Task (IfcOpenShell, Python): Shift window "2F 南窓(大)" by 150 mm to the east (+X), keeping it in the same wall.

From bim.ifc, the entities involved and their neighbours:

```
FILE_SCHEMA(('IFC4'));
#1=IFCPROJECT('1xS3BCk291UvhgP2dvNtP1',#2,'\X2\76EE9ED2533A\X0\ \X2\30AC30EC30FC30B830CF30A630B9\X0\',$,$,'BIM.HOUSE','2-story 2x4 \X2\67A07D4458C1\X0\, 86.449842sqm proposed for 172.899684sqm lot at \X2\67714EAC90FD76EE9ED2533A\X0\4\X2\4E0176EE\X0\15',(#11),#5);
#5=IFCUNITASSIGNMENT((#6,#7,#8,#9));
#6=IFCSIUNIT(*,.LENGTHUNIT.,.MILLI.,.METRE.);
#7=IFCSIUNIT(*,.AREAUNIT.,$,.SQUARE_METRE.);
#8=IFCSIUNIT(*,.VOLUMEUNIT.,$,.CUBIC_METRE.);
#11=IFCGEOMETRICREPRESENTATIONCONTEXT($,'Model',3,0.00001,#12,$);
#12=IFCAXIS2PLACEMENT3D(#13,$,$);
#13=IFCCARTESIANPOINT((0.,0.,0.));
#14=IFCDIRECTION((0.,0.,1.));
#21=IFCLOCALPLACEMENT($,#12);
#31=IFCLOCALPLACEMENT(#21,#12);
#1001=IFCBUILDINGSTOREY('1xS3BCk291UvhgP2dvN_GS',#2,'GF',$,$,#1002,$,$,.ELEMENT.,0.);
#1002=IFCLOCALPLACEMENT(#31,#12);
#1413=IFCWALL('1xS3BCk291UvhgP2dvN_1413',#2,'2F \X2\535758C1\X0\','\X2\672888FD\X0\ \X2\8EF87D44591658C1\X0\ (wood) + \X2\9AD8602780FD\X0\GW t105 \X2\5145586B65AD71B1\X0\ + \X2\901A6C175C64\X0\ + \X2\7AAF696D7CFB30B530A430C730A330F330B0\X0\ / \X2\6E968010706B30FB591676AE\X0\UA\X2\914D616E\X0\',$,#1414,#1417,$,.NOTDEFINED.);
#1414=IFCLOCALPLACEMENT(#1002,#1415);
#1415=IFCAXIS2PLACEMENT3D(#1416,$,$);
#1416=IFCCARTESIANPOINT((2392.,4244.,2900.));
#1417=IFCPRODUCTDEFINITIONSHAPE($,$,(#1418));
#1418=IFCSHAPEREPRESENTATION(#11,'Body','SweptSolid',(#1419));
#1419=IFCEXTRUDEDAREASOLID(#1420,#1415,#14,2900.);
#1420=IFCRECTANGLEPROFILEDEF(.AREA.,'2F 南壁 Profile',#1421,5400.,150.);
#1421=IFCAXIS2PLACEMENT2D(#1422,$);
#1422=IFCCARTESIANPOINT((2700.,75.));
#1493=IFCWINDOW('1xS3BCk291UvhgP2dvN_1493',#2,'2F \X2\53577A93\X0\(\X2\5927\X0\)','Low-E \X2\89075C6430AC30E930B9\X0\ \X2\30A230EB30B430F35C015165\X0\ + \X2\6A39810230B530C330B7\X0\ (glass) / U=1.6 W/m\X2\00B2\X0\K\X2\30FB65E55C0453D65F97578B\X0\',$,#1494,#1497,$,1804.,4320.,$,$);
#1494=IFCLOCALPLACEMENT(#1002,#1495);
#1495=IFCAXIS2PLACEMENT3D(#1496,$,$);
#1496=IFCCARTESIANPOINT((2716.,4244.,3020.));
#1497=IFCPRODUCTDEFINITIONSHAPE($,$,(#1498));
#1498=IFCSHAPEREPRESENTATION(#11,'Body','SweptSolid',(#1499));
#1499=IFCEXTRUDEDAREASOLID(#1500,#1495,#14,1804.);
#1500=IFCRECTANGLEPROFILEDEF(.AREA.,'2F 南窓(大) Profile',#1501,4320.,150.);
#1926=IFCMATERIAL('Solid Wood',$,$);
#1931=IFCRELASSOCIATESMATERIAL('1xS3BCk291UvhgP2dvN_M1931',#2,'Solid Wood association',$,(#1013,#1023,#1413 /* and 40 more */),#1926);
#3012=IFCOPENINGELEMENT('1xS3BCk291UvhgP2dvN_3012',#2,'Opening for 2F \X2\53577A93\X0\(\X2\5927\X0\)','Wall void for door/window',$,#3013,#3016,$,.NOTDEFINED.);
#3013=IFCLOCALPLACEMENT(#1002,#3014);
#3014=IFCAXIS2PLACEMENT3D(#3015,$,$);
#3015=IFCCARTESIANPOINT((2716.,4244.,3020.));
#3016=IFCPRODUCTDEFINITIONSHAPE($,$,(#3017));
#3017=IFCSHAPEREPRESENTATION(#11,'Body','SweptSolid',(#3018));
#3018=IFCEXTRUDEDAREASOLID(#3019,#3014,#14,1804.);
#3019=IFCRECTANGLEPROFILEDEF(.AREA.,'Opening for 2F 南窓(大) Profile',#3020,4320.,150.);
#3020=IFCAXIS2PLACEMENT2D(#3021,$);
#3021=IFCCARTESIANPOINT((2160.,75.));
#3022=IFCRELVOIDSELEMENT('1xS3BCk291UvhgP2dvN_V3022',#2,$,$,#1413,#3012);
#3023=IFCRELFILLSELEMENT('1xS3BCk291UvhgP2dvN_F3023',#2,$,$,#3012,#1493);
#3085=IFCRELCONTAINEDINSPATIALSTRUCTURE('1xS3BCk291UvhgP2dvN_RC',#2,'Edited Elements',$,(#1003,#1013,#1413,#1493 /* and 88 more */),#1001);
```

```python
import ifcopenshell
import ifcopenshell.api.geometry
import ifcopenshell.util.placement
import ifcopenshell.util.unit

model = ifcopenshell.open("bim.ifc")
unit_scale = ifcopenshell.util.unit.calculate_unit_scale(model)

window = model.by_guid("1xS3BCk291UvhgP2dvN_1493")
opening = window.FillsVoids[0].RelatingOpeningElement
wall = opening.VoidsElements[0].RelatingBuildingElement

wall_matrix = ifcopenshell.util.placement.get_local_placement(wall.ObjectPlacement)
shift = wall_matrix[:3, 0] * 0.15 / unit_scale
before = ifcopenshell.util.placement.get_local_placement(window.ObjectPlacement)[:3, 3].copy()

# The window is not placed relative to its opening, so move both.
for product in (opening, window):
    matrix = ifcopenshell.util.placement.get_local_placement(product.ObjectPlacement)
    matrix[:3, 3] += shift
    ifcopenshell.api.geometry.edit_object_placement(model, product=product, matrix=matrix, is_si=False)

after = ifcopenshell.util.placement.get_local_placement(window.ObjectPlacement)[:3, 3]
print("window moved by", (after - before).round(3) + 0.0)

model.write("bim_rev.ifc")
```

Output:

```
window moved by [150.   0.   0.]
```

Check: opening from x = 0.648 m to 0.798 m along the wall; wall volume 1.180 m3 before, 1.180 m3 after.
